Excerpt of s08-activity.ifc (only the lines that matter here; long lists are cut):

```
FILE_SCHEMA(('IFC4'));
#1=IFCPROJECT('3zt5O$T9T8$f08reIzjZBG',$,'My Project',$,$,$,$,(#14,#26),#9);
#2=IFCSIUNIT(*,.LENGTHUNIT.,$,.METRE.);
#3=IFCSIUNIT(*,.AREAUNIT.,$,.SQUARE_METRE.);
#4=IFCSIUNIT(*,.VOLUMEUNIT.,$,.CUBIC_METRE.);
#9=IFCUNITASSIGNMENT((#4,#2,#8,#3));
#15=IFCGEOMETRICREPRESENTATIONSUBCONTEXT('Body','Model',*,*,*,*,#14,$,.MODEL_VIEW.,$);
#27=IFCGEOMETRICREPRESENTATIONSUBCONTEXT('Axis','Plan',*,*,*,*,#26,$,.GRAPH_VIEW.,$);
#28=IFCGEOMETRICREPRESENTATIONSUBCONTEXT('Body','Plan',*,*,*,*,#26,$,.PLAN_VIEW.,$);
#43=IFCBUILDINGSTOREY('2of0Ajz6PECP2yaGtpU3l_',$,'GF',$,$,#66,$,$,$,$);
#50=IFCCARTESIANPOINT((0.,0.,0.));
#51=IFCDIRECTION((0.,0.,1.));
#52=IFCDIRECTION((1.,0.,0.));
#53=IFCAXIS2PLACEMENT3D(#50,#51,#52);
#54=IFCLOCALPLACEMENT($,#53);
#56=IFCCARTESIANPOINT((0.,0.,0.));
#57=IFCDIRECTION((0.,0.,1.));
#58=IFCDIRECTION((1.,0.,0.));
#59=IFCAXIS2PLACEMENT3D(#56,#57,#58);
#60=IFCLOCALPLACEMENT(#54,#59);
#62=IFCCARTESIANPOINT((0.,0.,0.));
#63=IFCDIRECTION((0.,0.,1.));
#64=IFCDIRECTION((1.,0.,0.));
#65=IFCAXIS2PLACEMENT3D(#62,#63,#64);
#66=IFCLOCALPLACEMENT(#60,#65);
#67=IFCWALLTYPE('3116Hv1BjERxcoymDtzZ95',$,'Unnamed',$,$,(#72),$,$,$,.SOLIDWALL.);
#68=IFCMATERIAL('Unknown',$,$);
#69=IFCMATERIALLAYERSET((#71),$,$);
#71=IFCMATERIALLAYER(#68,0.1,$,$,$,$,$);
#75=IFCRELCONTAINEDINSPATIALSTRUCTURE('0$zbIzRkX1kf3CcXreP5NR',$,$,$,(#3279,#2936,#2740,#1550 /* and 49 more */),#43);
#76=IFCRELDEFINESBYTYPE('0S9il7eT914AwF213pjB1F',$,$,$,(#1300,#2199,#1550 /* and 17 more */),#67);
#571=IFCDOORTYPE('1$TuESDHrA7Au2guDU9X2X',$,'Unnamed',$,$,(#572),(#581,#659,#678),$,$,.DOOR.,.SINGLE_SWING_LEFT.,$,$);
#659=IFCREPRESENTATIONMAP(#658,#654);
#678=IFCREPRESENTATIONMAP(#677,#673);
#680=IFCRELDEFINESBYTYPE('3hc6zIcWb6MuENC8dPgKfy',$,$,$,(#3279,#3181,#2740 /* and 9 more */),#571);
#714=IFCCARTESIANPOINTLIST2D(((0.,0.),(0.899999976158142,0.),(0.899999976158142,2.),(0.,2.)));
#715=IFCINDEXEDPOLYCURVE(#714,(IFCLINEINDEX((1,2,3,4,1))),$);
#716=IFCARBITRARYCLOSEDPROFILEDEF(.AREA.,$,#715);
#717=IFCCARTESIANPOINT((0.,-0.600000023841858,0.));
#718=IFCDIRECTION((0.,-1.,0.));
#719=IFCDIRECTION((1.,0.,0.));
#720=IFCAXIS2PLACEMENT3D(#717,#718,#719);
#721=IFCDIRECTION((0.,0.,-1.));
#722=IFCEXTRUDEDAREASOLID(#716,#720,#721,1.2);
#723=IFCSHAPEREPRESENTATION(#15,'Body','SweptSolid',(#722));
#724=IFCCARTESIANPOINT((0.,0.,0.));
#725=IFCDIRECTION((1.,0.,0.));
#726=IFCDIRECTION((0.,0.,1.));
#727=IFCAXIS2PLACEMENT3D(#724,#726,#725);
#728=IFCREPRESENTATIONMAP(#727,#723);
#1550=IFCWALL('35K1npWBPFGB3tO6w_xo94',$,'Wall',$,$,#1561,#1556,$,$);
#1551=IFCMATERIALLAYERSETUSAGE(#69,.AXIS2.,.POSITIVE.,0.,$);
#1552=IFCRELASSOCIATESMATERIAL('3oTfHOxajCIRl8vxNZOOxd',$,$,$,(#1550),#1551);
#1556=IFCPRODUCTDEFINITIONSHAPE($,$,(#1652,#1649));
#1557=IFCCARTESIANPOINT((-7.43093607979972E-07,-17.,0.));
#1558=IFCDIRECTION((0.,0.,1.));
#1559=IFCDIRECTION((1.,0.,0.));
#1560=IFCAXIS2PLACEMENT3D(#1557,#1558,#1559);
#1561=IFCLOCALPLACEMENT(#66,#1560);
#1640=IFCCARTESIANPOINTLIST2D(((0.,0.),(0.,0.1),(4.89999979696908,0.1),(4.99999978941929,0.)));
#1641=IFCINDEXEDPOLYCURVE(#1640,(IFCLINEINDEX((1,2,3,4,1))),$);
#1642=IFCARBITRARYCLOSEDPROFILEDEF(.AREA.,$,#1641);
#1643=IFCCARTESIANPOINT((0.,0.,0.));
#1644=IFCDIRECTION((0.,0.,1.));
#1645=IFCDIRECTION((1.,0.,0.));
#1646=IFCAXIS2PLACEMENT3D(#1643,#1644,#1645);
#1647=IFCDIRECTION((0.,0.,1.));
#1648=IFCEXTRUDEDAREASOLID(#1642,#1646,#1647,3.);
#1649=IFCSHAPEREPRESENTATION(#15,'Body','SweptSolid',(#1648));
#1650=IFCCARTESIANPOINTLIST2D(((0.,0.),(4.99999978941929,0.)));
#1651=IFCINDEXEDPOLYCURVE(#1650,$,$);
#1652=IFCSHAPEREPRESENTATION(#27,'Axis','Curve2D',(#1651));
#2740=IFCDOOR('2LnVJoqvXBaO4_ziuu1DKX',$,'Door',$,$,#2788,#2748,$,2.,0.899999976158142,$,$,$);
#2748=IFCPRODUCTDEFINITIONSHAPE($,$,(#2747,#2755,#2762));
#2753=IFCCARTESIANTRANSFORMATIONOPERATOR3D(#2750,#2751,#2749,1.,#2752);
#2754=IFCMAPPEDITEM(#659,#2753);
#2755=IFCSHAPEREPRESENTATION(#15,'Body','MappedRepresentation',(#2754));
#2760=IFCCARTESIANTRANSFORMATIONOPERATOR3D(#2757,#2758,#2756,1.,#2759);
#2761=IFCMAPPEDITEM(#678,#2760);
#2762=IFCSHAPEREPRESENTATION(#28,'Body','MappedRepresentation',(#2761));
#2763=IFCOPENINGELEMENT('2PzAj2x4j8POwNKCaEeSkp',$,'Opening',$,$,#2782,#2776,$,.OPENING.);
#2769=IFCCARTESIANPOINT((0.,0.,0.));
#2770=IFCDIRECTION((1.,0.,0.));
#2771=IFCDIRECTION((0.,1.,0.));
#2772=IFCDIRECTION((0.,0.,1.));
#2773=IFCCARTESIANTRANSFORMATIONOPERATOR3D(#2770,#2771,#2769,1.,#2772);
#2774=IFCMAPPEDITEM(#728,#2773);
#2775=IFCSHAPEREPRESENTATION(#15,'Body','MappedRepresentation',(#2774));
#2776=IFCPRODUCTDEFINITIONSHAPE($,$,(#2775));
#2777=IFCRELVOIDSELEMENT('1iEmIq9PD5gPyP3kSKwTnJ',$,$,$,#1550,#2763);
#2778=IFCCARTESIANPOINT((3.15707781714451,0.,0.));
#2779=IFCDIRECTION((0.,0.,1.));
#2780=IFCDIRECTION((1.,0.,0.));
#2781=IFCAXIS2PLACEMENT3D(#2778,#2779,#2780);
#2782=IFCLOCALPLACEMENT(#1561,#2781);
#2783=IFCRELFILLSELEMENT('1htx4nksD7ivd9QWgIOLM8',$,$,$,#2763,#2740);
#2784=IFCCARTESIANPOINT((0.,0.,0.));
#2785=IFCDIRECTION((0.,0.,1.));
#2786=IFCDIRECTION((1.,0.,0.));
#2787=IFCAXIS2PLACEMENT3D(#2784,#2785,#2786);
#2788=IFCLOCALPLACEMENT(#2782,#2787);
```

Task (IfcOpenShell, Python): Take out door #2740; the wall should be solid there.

```python
import ifcopenshell
import ifcopenshell.api.feature
import ifcopenshell.api.root
import ifcopenshell.geom
import ifcopenshell.util.shape

model = ifcopenshell.open("s08-activity.ifc")
settings = ifcopenshell.geom.settings()


def volume(element):
    """Net volume in cubic metres, openings subtracted."""
    shape = ifcopenshell.geom.create_shape(settings, element)
    return ifcopenshell.util.shape.get_volume(shape.geometry)


door = model.by_id(2740)
opening = door.FillsVoids[0].RelatingOpeningElement
wall = opening.VoidsElements[0].RelatingBuildingElement
before = volume(wall)

ifcopenshell.api.root.remove_product(model, product=door)
ifcopenshell.api.feature.remove_feature(model, feature=opening)

after = volume(wall)

print(f"wall volume {before:.3f} -> {after:.3f} m3")

model.write("s08-activity_v2.ifc")
```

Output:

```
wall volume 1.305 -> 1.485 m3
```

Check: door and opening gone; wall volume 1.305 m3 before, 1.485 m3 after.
